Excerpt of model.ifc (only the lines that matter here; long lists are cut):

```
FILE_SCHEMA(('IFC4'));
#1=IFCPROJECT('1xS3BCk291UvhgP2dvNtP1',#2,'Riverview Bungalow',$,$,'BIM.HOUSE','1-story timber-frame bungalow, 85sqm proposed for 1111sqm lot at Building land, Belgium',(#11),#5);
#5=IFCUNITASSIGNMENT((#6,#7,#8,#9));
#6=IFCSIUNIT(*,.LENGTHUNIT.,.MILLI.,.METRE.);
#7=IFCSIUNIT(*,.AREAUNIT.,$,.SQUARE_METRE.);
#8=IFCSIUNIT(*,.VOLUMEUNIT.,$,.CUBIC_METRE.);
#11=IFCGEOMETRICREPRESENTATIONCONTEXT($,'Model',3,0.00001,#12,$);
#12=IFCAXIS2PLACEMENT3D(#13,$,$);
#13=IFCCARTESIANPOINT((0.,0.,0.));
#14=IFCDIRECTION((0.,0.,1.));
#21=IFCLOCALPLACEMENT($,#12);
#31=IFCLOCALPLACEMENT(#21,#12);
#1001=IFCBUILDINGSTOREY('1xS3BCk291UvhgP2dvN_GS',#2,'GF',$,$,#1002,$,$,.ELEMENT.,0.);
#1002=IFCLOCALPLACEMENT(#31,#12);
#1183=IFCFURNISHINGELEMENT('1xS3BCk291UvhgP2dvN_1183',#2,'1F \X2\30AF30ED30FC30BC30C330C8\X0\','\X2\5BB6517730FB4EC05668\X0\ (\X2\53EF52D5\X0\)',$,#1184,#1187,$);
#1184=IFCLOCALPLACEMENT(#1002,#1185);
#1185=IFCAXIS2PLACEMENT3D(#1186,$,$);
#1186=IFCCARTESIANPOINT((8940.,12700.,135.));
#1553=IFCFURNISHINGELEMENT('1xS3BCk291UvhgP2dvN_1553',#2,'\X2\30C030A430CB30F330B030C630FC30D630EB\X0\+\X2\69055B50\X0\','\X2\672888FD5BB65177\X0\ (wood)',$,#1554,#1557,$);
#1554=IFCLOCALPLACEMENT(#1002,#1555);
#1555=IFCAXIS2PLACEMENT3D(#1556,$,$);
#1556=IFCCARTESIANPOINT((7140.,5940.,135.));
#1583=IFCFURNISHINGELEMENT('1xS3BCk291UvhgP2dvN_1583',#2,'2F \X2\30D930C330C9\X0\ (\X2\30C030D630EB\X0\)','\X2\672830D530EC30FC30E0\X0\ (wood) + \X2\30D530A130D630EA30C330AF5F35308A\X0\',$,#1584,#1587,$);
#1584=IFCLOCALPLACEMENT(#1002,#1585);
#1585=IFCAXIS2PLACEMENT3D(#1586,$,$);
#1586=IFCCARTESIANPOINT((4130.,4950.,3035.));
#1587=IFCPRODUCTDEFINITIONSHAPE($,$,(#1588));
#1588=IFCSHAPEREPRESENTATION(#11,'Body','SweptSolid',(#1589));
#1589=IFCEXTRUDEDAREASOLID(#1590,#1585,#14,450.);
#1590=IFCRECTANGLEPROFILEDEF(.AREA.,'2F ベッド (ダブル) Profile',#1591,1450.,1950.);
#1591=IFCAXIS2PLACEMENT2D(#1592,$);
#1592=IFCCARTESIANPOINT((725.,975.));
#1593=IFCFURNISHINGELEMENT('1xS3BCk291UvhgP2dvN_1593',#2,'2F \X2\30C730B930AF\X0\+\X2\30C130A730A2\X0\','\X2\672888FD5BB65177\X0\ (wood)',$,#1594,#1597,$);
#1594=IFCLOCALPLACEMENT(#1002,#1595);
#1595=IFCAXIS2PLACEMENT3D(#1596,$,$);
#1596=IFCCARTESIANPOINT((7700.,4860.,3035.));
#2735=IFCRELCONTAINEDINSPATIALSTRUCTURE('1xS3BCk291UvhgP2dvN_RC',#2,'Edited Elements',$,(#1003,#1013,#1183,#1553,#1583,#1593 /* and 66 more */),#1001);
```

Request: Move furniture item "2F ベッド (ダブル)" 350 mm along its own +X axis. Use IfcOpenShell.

```python
import ifcopenshell
import ifcopenshell.api.geometry
import ifcopenshell.util.placement
import ifcopenshell.util.unit

model = ifcopenshell.open("model.ifc")
unit_scale = ifcopenshell.util.unit.calculate_unit_scale(model)

item = model.by_guid("1xS3BCk291UvhgP2dvN_1583")
matrix = ifcopenshell.util.placement.get_local_placement(item.ObjectPlacement)
matrix[:3, 3] += matrix[:3, 0] * 0.35 / unit_scale
ifcopenshell.api.geometry.edit_object_placement(model, product=item, matrix=matrix, is_si=False)

print(ifcopenshell.util.placement.get_local_placement(item.ObjectPlacement).round(3) + 0.0)

model.write("model-out.ifc")
```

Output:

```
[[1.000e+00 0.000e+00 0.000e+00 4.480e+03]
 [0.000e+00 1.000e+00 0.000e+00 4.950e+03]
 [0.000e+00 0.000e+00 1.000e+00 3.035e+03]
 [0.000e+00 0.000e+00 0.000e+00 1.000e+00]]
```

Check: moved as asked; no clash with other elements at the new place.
